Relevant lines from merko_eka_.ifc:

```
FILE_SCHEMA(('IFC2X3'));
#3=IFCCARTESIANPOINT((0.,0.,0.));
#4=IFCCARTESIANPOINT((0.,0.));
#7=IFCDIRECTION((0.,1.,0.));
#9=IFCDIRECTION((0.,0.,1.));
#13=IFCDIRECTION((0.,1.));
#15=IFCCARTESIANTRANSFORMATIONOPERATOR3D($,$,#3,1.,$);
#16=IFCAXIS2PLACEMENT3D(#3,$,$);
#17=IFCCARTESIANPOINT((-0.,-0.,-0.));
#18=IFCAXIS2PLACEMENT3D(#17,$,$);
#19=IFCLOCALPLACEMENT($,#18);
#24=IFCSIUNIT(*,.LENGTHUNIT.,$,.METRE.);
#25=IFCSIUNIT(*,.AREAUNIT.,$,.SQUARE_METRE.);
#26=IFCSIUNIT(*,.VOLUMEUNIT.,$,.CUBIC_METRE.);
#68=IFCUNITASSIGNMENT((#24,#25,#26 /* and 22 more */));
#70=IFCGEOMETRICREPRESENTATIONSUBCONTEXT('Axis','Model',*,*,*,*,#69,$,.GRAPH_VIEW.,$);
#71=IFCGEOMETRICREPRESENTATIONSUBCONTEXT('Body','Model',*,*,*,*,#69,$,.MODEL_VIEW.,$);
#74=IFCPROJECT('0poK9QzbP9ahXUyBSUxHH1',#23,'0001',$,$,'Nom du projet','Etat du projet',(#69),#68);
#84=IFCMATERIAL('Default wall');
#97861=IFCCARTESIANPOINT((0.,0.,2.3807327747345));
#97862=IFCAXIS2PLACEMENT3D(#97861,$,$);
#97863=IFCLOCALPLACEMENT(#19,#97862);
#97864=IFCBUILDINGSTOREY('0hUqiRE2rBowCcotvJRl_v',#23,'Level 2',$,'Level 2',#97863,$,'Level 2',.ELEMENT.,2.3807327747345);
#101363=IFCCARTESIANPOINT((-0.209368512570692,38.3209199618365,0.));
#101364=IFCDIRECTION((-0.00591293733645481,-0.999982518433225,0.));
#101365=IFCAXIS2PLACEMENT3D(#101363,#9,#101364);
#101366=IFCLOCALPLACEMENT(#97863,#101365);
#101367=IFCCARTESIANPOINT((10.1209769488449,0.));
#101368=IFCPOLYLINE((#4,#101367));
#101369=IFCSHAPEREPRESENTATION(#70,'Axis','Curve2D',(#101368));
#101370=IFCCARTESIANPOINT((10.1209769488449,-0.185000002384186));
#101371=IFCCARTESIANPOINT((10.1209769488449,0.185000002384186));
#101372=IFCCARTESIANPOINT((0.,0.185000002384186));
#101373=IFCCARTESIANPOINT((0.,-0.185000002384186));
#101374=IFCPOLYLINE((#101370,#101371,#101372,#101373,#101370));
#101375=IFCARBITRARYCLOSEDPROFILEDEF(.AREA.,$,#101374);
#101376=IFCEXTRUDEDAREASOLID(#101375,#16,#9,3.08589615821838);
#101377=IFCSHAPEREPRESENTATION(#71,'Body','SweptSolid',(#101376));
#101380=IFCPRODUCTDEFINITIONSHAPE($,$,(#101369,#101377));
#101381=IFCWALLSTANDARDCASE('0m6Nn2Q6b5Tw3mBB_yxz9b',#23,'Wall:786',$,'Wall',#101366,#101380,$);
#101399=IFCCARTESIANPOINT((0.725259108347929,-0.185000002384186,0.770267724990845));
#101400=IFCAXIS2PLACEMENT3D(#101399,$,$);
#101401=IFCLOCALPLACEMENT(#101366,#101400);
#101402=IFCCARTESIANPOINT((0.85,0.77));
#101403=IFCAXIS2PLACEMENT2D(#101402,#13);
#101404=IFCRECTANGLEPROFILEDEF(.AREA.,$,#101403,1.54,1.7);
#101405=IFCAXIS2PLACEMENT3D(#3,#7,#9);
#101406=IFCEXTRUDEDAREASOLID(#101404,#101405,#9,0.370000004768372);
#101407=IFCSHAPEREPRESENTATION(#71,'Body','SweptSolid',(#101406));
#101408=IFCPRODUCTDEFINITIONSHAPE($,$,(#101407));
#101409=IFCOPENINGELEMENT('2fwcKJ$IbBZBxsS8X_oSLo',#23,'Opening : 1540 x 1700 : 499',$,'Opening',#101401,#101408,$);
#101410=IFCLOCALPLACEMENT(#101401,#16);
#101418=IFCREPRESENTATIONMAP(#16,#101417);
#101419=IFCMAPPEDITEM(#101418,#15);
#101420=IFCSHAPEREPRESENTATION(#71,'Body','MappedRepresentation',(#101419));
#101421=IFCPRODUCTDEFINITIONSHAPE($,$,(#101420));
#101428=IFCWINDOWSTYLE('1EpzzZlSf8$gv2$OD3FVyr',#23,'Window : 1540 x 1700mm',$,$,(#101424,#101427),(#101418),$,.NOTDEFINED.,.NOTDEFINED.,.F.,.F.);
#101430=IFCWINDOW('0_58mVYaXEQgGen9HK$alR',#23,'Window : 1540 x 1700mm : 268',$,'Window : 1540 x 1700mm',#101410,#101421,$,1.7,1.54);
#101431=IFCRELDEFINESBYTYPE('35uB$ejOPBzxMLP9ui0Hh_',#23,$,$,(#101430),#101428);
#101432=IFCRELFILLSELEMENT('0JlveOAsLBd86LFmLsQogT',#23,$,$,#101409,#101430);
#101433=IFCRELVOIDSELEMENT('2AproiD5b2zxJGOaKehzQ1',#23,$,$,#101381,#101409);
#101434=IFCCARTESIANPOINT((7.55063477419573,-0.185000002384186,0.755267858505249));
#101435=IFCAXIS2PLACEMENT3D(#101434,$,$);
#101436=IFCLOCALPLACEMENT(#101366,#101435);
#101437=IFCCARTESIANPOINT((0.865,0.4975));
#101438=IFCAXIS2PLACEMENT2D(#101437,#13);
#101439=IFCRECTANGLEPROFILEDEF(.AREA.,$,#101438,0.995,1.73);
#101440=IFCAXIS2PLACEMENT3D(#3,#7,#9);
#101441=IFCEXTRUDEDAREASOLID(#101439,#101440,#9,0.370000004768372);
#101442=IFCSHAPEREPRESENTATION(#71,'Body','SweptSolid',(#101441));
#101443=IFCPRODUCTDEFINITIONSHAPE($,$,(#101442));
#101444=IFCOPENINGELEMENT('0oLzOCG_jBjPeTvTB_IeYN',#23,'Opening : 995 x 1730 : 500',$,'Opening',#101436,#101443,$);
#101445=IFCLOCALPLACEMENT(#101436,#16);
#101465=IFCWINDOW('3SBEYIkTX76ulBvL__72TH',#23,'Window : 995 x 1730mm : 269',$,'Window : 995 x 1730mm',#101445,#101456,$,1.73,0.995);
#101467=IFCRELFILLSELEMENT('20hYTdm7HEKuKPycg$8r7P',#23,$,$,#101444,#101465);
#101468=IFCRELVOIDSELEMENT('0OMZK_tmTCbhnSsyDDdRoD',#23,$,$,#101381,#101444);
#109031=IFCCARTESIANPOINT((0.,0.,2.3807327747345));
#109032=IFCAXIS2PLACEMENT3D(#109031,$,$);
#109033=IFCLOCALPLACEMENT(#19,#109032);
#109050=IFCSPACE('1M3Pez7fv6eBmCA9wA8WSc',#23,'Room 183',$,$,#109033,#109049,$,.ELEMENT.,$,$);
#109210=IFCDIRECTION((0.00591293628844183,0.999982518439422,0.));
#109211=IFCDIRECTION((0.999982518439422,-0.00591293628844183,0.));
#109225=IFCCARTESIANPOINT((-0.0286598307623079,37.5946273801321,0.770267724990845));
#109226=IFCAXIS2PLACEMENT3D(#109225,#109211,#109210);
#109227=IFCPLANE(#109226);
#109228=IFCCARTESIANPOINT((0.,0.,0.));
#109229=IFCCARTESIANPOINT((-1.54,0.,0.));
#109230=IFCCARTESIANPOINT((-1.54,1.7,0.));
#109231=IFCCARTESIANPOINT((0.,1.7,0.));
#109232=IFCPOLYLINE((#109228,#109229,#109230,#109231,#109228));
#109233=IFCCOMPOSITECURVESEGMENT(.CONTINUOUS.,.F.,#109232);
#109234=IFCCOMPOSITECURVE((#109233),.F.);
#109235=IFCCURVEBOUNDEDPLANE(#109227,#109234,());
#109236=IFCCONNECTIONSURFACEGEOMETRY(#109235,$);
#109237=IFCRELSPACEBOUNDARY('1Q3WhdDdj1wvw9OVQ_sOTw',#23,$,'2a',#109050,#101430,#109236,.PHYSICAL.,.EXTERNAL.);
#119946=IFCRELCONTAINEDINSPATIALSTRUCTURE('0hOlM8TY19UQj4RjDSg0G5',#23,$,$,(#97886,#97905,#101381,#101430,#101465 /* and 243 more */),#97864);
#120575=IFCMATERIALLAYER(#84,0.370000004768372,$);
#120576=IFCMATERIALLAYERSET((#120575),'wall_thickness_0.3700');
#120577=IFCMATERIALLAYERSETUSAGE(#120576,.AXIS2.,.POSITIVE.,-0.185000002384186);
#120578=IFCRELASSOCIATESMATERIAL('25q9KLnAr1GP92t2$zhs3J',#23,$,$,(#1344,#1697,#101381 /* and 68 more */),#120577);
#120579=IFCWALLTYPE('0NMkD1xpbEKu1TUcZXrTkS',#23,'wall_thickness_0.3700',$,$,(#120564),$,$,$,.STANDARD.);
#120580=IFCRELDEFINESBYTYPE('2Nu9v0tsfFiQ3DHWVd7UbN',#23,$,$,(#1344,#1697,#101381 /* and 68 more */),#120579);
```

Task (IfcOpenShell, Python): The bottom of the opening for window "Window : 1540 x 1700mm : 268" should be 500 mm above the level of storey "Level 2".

```python
import numpy as np
import ifcopenshell
import ifcopenshell.api.geometry
import ifcopenshell.geom
import ifcopenshell.util.element
import ifcopenshell.util.placement
import ifcopenshell.util.shape
import ifcopenshell.util.unit

model = ifcopenshell.open("merko_eka_.ifc")
unit_scale = ifcopenshell.util.unit.calculate_unit_scale(model)

window = model.by_guid("0_58mVYaXEQgGen9HK$alR")
opening = window.FillsVoids[0].RelatingOpeningElement
storey = ifcopenshell.util.element.get_container(window, ifc_class="IfcBuildingStorey")
level = ifcopenshell.util.placement.get_local_placement(storey.ObjectPlacement)[2, 3]

# The opening's origin need not be at the sill, so measure its lowest point.
shape = ifcopenshell.geom.create_shape(ifcopenshell.geom.settings(), opening)
bottom = ifcopenshell.util.shape.get_shape_bottom_elevation(shape, shape.geometry) / unit_scale
dz = level + 0.5 / unit_scale - bottom

shift = np.array([0.0, 0.0, dz])
# The window is placed relative to its opening, so it follows when the opening moves.
matrix = ifcopenshell.util.placement.get_local_placement(opening.ObjectPlacement)
matrix[:3, 3] += shift
ifcopenshell.api.geometry.edit_object_placement(
    model, product=opening, matrix=matrix, is_si=False, should_transform_children=True
)

# Space boundary surfaces are stored in each space's coordinates; move them too.
for rel in window.ProvidesBoundaries:
    if not rel.ConnectionGeometry:
        continue
    surface = rel.ConnectionGeometry.SurfaceOnRelatingElement.BasisSurface
    space_matrix = ifcopenshell.util.placement.get_local_placement(rel.RelatingSpace.ObjectPlacement)
    point = np.array(surface.Position.Location.Coordinates) + space_matrix[:3, :3].T @ shift
    surface.Position = model.createIfcAxis2Placement3D(
        model.createIfcCartesianPoint(point.tolist()), surface.Position.Axis, surface.Position.RefDirection
    )

print(f"moved by {dz * unit_scale:+.3f} m")

model.write("merko_eka__v2.ifc")
```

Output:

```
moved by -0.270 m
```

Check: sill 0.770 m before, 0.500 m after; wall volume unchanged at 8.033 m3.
